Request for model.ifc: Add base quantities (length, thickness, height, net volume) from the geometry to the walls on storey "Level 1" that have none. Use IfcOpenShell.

First a look at what the model holds.

```python
import ifcopenshell
import ifcopenshell.util.element
import ifcopenshell.util.unit

model = ifcopenshell.open("model.ifc")
print(model.schema)
for unit_type in ("LENGTHUNIT", "AREAUNIT", "VOLUMEUNIT"):
    print(unit_type, ifcopenshell.util.unit.calculate_unit_scale(model, unit_type))
storey = next(s for s in model.by_type("IfcBuildingStorey") if s.Name == "Level 1")
walls = [e for e in ifcopenshell.util.element.get_decomposition(storey) if e.is_a("IfcWall")]
for e in sorted(walls, key=lambda e: e.id()):
    print(e.id(), e.is_a(), e.Name, list(ifcopenshell.util.element.get_psets(e, qtos_only=True)), sep=" | ")
```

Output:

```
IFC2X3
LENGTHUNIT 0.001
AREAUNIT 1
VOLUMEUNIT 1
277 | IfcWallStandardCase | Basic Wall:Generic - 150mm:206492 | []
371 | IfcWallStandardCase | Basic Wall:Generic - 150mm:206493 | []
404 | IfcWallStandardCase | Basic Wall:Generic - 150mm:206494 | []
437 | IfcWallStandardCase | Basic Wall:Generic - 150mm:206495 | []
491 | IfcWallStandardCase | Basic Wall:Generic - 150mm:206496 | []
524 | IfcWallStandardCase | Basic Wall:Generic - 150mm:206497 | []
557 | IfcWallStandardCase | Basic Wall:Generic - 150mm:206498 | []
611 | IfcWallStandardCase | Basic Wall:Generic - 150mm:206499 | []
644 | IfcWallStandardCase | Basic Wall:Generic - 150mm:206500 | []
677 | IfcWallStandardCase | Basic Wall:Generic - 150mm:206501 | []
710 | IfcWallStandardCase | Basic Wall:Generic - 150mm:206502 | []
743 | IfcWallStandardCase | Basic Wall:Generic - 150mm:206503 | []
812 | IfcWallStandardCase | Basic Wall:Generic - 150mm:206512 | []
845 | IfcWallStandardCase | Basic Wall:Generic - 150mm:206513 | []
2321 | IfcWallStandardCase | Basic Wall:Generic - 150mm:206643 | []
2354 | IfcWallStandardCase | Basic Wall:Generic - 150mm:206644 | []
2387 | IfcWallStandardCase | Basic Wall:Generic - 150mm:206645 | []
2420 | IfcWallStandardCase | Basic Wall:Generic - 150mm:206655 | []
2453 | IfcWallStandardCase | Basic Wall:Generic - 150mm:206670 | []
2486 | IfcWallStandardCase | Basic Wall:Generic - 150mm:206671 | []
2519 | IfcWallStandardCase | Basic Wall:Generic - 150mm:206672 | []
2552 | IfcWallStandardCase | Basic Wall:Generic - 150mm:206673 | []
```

```python
import ifcopenshell
import ifcopenshell.api.pset
import ifcopenshell.geom
import ifcopenshell.util.element
import ifcopenshell.util.shape
import ifcopenshell.util.unit

model = ifcopenshell.open("model.ifc")
unit_scale = ifcopenshell.util.unit.calculate_unit_scale(model)
volume_scale = ifcopenshell.util.unit.calculate_unit_scale(model, "VOLUMEUNIT")
settings = ifcopenshell.geom.settings()

storey = next(s for s in model.by_type("IfcBuildingStorey") if s.Name == "Level 1")
walls = [e for e in ifcopenshell.util.element.get_decomposition(storey) if e.is_a("IfcWall")]

for e in sorted(walls, key=lambda e: e.id()):
    if ifcopenshell.util.element.get_psets(e, qtos_only=True, should_inherit=False):
        continue
    # Geometry comes back in metres, in the element's own axes.
    shape = ifcopenshell.geom.create_shape(settings, e)
    values = {
        "Length": ifcopenshell.util.shape.get_x(shape.geometry) / unit_scale,
        "Width": ifcopenshell.util.shape.get_y(shape.geometry) / unit_scale,
        "Height": ifcopenshell.util.shape.get_z(shape.geometry) / unit_scale,
        "NetVolume": ifcopenshell.util.shape.get_volume(shape.geometry) / volume_scale,
    }
    qto = ifcopenshell.api.pset.add_qto(model, product=e, name="BaseQuantities")
    ifcopenshell.api.pset.edit_qto(model, qto=qto, properties=values)
    print(e.id(), {k: round(v, 3) for k, v in values.items()})

model.write("model_v2.ifc")
```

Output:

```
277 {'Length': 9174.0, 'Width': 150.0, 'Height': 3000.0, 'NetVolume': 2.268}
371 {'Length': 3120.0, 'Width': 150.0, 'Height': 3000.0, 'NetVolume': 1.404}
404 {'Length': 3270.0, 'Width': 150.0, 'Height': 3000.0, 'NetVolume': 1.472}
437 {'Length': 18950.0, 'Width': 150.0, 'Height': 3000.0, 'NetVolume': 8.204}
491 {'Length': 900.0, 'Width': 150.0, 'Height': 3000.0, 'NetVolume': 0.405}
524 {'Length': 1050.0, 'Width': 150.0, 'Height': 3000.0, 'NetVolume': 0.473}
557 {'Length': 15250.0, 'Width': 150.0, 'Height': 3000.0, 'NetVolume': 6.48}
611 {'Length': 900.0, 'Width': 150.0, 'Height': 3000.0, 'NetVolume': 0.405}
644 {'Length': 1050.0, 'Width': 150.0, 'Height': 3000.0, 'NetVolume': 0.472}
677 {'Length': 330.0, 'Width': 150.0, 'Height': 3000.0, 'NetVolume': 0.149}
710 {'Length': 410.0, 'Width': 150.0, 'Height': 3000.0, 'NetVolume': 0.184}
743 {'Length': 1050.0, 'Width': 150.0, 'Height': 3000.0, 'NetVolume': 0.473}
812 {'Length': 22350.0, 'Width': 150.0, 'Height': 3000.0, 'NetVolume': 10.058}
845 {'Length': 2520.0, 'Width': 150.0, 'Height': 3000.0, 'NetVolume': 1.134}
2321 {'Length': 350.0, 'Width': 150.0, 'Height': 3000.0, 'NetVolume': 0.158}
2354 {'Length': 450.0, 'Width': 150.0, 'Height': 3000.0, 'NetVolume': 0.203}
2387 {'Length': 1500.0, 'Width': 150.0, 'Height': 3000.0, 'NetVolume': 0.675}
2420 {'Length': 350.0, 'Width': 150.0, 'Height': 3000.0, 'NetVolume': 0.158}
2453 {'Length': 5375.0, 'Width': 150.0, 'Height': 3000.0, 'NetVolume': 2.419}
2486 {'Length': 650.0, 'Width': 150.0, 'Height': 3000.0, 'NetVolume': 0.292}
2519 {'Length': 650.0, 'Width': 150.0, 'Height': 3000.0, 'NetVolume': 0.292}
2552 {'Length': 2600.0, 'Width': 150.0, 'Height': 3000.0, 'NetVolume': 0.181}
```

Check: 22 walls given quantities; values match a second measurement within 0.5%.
